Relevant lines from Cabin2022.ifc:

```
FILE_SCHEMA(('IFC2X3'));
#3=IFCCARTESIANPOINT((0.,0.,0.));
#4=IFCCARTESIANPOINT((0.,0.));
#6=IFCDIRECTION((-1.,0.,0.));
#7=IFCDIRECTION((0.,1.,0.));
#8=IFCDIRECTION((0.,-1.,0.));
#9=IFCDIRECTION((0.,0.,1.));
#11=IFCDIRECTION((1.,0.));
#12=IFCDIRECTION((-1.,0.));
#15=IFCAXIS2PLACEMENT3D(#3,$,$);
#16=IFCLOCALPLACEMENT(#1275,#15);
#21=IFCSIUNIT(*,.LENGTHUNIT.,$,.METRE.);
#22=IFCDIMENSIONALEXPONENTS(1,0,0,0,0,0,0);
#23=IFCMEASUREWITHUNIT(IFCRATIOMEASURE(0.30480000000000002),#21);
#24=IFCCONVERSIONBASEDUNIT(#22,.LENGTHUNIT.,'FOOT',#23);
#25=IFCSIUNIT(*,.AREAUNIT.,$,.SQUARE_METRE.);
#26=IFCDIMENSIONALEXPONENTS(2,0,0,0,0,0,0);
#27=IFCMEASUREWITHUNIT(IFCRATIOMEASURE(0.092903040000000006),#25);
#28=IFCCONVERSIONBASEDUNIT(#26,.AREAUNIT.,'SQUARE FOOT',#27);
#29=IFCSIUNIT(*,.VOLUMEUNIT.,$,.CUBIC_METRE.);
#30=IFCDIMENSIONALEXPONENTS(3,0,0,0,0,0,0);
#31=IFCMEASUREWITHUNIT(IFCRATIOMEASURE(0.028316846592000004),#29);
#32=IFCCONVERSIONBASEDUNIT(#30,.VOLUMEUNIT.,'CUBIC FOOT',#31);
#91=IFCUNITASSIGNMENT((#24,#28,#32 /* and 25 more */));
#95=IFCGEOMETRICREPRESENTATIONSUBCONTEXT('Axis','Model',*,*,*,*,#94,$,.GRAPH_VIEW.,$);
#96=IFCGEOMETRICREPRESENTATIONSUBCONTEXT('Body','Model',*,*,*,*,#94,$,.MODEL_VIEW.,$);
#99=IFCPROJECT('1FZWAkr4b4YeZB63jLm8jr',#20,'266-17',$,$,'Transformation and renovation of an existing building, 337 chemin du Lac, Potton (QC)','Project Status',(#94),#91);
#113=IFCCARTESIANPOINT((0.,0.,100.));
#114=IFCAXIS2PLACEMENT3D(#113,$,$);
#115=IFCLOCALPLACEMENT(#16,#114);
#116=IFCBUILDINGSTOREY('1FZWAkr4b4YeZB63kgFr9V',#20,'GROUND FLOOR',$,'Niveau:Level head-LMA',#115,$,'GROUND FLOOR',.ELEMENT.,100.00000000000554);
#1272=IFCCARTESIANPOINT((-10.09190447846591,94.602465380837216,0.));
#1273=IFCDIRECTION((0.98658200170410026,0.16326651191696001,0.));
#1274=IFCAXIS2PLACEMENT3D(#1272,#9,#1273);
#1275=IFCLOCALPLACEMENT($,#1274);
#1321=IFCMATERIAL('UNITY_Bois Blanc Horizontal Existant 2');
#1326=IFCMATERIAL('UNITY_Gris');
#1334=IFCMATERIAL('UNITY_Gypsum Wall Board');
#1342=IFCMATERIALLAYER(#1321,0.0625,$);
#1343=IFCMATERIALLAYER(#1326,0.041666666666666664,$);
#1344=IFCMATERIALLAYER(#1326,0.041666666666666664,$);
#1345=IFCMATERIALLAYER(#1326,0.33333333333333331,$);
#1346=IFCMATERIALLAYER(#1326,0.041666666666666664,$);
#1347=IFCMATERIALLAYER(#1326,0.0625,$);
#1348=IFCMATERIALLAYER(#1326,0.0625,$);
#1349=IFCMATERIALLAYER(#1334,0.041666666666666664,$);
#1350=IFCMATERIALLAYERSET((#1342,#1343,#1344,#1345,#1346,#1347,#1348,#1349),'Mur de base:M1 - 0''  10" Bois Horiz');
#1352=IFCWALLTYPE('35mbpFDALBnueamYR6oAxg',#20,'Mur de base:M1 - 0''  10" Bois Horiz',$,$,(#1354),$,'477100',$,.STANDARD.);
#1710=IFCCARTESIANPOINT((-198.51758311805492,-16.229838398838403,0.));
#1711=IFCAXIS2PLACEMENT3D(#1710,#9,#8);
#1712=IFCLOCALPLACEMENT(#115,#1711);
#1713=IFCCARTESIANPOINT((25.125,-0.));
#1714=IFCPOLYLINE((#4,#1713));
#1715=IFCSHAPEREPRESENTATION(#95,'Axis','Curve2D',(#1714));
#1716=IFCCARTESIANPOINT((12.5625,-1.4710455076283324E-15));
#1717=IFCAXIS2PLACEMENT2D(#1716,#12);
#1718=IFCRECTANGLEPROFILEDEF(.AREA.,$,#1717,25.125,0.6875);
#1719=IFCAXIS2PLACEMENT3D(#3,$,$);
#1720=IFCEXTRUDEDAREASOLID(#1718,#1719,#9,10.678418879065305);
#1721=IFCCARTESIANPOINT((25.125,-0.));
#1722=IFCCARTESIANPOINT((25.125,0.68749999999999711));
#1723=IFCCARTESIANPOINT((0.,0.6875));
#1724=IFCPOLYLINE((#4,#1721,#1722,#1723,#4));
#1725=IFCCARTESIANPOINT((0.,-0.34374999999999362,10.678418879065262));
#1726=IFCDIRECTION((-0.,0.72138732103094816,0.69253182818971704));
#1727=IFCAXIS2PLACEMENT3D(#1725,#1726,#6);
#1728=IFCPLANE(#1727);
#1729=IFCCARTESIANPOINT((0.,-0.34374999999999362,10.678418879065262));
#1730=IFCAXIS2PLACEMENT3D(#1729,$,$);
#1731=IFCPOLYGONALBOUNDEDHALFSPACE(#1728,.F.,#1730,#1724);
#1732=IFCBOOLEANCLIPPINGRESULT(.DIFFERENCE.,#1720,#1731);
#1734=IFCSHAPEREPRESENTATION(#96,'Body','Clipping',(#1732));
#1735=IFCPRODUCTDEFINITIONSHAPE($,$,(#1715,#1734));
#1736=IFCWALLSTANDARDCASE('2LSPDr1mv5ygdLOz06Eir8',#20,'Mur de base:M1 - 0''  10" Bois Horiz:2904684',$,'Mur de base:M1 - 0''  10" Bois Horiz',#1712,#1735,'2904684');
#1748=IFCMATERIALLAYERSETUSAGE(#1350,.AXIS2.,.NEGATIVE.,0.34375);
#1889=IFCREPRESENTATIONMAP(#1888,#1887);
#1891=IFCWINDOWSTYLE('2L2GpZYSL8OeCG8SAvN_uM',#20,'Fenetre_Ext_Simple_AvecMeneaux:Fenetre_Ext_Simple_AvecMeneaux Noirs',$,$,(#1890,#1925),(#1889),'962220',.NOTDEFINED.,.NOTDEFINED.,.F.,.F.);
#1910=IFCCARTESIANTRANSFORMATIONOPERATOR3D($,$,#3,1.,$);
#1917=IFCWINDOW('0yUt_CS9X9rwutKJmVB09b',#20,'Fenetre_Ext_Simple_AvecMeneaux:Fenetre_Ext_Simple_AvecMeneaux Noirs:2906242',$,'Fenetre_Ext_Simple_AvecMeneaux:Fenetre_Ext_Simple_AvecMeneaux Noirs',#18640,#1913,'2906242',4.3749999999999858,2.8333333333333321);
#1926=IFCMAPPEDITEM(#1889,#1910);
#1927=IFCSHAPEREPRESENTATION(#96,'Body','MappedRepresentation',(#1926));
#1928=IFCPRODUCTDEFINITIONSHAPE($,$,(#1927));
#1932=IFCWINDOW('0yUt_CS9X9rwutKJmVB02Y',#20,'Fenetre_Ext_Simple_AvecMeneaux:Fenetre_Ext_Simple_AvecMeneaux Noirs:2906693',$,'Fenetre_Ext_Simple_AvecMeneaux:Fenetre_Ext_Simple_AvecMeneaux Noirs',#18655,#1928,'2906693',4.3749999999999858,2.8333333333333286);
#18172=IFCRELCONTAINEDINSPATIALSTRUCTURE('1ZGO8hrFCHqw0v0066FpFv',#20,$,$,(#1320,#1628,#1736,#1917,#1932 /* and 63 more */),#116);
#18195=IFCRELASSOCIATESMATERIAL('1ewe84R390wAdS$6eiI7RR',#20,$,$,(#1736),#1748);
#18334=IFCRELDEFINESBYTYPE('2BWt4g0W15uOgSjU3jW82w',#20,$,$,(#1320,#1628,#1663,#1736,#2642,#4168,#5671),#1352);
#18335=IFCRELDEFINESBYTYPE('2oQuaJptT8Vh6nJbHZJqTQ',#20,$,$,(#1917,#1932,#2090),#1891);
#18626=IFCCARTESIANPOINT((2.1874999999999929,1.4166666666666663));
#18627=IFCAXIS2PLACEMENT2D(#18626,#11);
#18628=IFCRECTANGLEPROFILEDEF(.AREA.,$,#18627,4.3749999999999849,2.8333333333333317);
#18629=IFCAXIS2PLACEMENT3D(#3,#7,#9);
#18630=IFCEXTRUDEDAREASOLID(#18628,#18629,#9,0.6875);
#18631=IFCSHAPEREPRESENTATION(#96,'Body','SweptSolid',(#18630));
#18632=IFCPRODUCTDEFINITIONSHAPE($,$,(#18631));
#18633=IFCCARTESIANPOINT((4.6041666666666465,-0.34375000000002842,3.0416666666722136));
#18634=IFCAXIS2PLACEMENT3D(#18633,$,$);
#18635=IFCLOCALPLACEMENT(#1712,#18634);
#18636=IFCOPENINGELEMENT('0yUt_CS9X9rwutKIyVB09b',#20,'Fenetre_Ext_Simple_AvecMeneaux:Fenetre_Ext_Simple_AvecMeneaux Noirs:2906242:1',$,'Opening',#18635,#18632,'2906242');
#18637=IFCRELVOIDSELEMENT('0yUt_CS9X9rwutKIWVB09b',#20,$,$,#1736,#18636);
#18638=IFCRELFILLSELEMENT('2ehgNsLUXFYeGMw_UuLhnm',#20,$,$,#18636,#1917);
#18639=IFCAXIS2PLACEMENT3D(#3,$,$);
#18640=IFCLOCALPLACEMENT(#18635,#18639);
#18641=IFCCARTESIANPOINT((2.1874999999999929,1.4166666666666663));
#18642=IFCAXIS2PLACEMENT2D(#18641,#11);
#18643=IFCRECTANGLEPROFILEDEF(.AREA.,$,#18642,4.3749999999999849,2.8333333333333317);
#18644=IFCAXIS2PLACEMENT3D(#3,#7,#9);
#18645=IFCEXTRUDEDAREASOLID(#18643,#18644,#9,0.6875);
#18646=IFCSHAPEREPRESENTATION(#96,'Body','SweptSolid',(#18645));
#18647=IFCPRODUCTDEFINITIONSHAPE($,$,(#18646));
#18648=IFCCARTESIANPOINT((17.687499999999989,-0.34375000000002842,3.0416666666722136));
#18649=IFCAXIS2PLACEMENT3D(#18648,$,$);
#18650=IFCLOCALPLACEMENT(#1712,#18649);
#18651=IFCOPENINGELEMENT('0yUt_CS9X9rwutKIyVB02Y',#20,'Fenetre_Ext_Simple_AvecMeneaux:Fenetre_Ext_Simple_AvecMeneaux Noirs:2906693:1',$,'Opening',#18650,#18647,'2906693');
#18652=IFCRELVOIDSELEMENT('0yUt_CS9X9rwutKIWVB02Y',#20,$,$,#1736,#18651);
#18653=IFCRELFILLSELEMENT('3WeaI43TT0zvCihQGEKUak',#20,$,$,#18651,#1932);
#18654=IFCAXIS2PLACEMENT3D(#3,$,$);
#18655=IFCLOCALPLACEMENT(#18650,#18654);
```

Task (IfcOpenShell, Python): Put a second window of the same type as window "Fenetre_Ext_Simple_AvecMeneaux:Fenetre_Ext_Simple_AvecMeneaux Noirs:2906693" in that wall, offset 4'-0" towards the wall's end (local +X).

```python
import ifcopenshell
import ifcopenshell.api.feature
import ifcopenshell.api.geometry
import ifcopenshell.api.root
import ifcopenshell.geom
import ifcopenshell.util.element
import ifcopenshell.util.placement
import ifcopenshell.util.shape
import ifcopenshell.util.unit

model = ifcopenshell.open("Cabin2022.ifc")
unit_scale = ifcopenshell.util.unit.calculate_unit_scale(model)
settings = ifcopenshell.geom.settings()


def volume(element):
    """Net volume in cubic metres, openings subtracted."""
    shape = ifcopenshell.geom.create_shape(settings, element)
    return ifcopenshell.util.shape.get_volume(shape.geometry)


def reuse_history(source, copy):
    """copy_class also copies each property set's owner history, people and application; keep the originals."""
    for rel in copy.IsDefinedBy:
        if rel.is_a("IfcRelDefinesByProperties") and (history := rel.RelatingPropertyDefinition.OwnerHistory):
            rel.RelatingPropertyDefinition.OwnerHistory = source.OwnerHistory
            ifcopenshell.util.element.remove_deep2(model, history)


window = model.by_guid("0yUt_CS9X9rwutKJmVB02Y")
opening = window.FillsVoids[0].RelatingOpeningElement
wall = opening.VoidsElements[0].RelatingBuildingElement
before = volume(wall)
shift = ifcopenshell.util.placement.get_local_placement(wall.ObjectPlacement)[:3, 0] * 48 * 0.0254 / unit_scale

# copy_class copies the void relationship, type, container and properties, but no geometry.
new_opening = ifcopenshell.api.root.copy_class(model, product=opening)
new_opening.Representation = ifcopenshell.util.element.copy_deep(
    model, opening.Representation, exclude=["IfcGeometricRepresentationContext", "IfcRepresentationMap"]
)
new_opening.Name = "Fenetre_Ext_Simple_AvecMeneaux:Fenetre_Ext_Simple_AvecMeneaux Noirs"
new_opening.Tag = None
new_window = ifcopenshell.api.root.copy_class(model, product=window)
new_window.Representation = ifcopenshell.util.element.copy_deep(
    model, window.Representation, exclude=["IfcGeometricRepresentationContext", "IfcRepresentationMap"]
)
new_window.Name = "Fenetre_Ext_Simple_AvecMeneaux:Fenetre_Ext_Simple_AvecMeneaux Noirs"
new_window.Tag = None
reuse_history(window, new_window)
fills = ifcopenshell.api.feature.add_filling(model, opening=new_opening, element=new_window)
fills.OwnerHistory = new_window.OwnerHistory  # required in IFC2X3

for old, new in ((opening, new_opening), (window, new_window)):
    matrix = ifcopenshell.util.placement.get_local_placement(old.ObjectPlacement)
    matrix[:3, 3] += shift
    ifcopenshell.api.geometry.edit_object_placement(model, product=new, matrix=matrix, is_si=False)

after = volume(wall)

print(f"wall volume {before:.3f} -> {after:.3f} m3")

model.write("Cabin2022_rev.ifc")
```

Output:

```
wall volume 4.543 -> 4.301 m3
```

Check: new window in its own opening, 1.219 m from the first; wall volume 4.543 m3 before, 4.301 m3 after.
